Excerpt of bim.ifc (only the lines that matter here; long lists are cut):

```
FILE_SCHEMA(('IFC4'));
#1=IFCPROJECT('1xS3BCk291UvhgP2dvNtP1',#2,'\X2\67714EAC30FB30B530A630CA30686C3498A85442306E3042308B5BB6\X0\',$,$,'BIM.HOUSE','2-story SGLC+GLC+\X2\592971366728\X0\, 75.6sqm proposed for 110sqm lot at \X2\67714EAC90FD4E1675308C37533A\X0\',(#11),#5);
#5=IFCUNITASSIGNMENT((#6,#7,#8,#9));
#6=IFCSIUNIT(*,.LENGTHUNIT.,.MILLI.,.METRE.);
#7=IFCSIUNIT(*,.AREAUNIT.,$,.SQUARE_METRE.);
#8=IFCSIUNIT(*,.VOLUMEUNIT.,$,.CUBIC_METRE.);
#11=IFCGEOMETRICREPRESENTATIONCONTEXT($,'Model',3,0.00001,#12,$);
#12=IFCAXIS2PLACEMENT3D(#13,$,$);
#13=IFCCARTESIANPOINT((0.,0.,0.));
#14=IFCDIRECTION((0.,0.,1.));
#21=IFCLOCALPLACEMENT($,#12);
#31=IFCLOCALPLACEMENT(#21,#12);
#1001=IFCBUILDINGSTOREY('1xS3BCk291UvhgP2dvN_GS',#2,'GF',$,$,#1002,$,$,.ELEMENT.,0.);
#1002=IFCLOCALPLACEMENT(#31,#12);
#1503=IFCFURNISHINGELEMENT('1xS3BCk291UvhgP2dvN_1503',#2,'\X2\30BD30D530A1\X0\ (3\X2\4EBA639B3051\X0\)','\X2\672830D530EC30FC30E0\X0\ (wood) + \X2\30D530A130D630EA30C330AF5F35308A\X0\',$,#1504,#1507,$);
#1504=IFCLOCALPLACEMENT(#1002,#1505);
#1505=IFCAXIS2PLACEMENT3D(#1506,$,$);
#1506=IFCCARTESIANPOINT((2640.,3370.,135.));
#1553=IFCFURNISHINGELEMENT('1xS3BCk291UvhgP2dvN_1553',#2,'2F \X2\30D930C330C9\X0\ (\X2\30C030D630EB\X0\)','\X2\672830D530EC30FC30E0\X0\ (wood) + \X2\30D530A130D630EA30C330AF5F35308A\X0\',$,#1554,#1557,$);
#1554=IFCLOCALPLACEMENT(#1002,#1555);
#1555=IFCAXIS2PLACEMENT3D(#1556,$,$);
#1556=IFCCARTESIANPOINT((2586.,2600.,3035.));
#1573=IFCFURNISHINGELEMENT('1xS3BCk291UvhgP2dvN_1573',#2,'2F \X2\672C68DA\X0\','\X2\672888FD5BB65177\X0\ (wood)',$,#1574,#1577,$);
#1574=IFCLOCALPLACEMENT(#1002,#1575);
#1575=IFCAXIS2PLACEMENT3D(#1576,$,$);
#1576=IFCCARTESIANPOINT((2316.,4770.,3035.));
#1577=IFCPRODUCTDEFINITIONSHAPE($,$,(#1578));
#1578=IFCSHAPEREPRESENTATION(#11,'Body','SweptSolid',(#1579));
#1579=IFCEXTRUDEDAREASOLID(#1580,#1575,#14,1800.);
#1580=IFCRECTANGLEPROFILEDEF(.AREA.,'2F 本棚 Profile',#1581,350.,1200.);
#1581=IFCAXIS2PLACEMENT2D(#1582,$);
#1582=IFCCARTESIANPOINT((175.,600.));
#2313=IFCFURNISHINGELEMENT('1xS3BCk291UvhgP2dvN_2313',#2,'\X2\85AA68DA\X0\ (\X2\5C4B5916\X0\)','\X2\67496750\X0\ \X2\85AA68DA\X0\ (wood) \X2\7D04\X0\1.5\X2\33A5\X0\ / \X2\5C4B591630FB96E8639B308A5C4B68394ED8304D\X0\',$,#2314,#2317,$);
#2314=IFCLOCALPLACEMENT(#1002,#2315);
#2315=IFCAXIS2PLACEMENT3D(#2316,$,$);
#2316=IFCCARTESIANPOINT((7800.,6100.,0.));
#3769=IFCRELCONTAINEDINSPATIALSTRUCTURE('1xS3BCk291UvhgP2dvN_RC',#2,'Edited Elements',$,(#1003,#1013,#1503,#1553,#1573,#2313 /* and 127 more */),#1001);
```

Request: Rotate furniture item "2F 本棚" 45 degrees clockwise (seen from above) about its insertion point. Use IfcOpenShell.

```python
import ifcopenshell
import ifcopenshell.api.geometry
import ifcopenshell.util.placement

model = ifcopenshell.open("bim.ifc")

item = model.by_guid("1xS3BCk291UvhgP2dvN_1573")
matrix = ifcopenshell.util.placement.get_local_placement(item.ObjectPlacement)
matrix = matrix @ ifcopenshell.util.placement.rotation(-45, "Z")
ifcopenshell.api.geometry.edit_object_placement(model, product=item, matrix=matrix, is_si=False)

print(ifcopenshell.util.placement.get_local_placement(item.ObjectPlacement).round(3) + 0.0)

model.write("bim_updated.ifc")
```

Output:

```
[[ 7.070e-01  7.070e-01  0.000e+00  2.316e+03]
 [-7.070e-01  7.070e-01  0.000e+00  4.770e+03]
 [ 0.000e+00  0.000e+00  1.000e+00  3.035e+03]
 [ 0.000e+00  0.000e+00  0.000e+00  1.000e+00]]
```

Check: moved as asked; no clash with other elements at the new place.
